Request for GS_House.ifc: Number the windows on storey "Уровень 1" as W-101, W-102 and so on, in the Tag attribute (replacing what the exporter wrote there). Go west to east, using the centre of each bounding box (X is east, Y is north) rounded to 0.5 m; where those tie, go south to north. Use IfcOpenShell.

First a look at what the model holds.

```python
import ifcopenshell
import ifcopenshell.util.element
import ifcopenshell.util.placement

model = ifcopenshell.open("GS_House.ifc")
print(model.schema)
storey = next(s for s in model.by_type("IfcBuildingStorey") if s.Name == "Уровень 1")
windows = [e for e in ifcopenshell.util.element.get_decomposition(storey) if e.is_a("IfcWindow")]
for e in sorted(windows, key=lambda e: e.id()):
    origin = ifcopenshell.util.placement.get_local_placement(e.ObjectPlacement)[:3, 3]
    print(e.id(), e.Tag, e.Name, origin.round(2) + 0.0, sep=" | ")
```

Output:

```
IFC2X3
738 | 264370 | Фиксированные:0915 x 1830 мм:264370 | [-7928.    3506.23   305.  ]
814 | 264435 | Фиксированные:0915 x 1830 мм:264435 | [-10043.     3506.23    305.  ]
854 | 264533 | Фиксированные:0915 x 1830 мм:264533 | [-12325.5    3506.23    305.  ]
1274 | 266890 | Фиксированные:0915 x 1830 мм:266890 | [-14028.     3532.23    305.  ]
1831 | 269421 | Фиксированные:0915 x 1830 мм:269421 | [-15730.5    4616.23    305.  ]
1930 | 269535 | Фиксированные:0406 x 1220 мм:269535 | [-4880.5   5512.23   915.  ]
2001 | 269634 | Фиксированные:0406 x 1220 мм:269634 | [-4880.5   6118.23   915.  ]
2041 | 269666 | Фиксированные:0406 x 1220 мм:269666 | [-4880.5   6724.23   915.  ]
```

```python
import ifcopenshell
import ifcopenshell.geom
import ifcopenshell.util.element
import ifcopenshell.util.shape

model = ifcopenshell.open("GS_House.ifc")
settings = ifcopenshell.geom.settings()
settings.set("use-world-coords", True)


def centre(element):
    shape = ifcopenshell.geom.create_shape(settings, element)
    return ifcopenshell.util.shape.get_bbox_centroid(shape.geometry)


storey = next(s for s in model.by_type("IfcBuildingStorey") if s.Name == "Уровень 1")
windows = [e for e in ifcopenshell.util.element.get_decomposition(storey) if e.is_a("IfcWindow")]

# Insertion points can sit at a corner or the storey origin, so sort by the geometry (in metres).
centres = {e: centre(e) for e in windows}
windows.sort(key=lambda e: (round(centres[e][0] / 0.5), centres[e][1]))

for i, e in enumerate(windows, start=1):
    number = f"W-1{i:02d}"
    e.Tag = number
    print(e.id(), number)

model.write("GS_House_updated.ifc")
```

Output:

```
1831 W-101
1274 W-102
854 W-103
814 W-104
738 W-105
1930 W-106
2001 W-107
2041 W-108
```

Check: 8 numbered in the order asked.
